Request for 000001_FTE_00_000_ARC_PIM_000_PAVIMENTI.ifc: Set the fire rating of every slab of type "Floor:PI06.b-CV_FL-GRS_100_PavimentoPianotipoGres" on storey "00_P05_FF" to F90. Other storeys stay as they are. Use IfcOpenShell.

First a look at what the model holds.

```python
import ifcopenshell
import ifcopenshell.util.element

model = ifcopenshell.open("000001_FTE_00_000_ARC_PIM_000_PAVIMENTI.ifc")
print(model.schema)
storey = next(s for s in model.by_type("IfcBuildingStorey") if s.Name == "00_P05_FF")
slabs = [e for e in ifcopenshell.util.element.get_decomposition(storey) if e.is_a("IfcSlab")]
seen = {}
for e in slabs:
    element_type = ifcopenshell.util.element.get_type(e)
    key = (element_type.Name if element_type != e and element_type else None, ifcopenshell.util.element.get_pset(e, "Pset_SlabCommon", "FireRating"))
    seen[key] = seen.get(key, 0) + 1
for (name, value), count in sorted(seen.items(), key=str):
    print(count, "x", name, "|", value)
```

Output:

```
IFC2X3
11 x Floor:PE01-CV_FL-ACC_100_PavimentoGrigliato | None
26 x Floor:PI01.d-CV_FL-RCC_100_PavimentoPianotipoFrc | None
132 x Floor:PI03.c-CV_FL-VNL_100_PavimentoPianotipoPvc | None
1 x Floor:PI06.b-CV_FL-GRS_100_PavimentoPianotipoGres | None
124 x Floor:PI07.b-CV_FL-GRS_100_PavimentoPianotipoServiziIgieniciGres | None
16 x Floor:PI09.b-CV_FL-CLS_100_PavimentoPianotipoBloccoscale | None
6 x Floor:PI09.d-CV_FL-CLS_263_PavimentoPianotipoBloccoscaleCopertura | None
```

```python
import ifcopenshell
import ifcopenshell.api.pset
import ifcopenshell.util.element

model = ifcopenshell.open("000001_FTE_00_000_ARC_PIM_000_PAVIMENTI.ifc")

storey = next(s for s in model.by_type("IfcBuildingStorey") if s.Name == "00_P05_FF")
slabs = [e for e in ifcopenshell.util.element.get_decomposition(storey) if e.is_a("IfcSlab")]

count = 0
for e in slabs:
    element_type = ifcopenshell.util.element.get_type(e)
    if element_type in (None, e) or element_type.Name != "Floor:PI06.b-CV_FL-GRS_100_PavimentoPianotipoGres":
        continue
    # add_pset returns the element's existing set when there is one.
    pset = ifcopenshell.api.pset.add_pset(model, product=e, name="Pset_SlabCommon")
    ifcopenshell.api.pset.edit_pset(model, pset=pset, properties={"FireRating": "F90"})
    count += 1

print(count, "slabs updated")

model.write("000001_FTE_00_000_ARC_PIM_000_PAVIMENTI-out.ifc")
```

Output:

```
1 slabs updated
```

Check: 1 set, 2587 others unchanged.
